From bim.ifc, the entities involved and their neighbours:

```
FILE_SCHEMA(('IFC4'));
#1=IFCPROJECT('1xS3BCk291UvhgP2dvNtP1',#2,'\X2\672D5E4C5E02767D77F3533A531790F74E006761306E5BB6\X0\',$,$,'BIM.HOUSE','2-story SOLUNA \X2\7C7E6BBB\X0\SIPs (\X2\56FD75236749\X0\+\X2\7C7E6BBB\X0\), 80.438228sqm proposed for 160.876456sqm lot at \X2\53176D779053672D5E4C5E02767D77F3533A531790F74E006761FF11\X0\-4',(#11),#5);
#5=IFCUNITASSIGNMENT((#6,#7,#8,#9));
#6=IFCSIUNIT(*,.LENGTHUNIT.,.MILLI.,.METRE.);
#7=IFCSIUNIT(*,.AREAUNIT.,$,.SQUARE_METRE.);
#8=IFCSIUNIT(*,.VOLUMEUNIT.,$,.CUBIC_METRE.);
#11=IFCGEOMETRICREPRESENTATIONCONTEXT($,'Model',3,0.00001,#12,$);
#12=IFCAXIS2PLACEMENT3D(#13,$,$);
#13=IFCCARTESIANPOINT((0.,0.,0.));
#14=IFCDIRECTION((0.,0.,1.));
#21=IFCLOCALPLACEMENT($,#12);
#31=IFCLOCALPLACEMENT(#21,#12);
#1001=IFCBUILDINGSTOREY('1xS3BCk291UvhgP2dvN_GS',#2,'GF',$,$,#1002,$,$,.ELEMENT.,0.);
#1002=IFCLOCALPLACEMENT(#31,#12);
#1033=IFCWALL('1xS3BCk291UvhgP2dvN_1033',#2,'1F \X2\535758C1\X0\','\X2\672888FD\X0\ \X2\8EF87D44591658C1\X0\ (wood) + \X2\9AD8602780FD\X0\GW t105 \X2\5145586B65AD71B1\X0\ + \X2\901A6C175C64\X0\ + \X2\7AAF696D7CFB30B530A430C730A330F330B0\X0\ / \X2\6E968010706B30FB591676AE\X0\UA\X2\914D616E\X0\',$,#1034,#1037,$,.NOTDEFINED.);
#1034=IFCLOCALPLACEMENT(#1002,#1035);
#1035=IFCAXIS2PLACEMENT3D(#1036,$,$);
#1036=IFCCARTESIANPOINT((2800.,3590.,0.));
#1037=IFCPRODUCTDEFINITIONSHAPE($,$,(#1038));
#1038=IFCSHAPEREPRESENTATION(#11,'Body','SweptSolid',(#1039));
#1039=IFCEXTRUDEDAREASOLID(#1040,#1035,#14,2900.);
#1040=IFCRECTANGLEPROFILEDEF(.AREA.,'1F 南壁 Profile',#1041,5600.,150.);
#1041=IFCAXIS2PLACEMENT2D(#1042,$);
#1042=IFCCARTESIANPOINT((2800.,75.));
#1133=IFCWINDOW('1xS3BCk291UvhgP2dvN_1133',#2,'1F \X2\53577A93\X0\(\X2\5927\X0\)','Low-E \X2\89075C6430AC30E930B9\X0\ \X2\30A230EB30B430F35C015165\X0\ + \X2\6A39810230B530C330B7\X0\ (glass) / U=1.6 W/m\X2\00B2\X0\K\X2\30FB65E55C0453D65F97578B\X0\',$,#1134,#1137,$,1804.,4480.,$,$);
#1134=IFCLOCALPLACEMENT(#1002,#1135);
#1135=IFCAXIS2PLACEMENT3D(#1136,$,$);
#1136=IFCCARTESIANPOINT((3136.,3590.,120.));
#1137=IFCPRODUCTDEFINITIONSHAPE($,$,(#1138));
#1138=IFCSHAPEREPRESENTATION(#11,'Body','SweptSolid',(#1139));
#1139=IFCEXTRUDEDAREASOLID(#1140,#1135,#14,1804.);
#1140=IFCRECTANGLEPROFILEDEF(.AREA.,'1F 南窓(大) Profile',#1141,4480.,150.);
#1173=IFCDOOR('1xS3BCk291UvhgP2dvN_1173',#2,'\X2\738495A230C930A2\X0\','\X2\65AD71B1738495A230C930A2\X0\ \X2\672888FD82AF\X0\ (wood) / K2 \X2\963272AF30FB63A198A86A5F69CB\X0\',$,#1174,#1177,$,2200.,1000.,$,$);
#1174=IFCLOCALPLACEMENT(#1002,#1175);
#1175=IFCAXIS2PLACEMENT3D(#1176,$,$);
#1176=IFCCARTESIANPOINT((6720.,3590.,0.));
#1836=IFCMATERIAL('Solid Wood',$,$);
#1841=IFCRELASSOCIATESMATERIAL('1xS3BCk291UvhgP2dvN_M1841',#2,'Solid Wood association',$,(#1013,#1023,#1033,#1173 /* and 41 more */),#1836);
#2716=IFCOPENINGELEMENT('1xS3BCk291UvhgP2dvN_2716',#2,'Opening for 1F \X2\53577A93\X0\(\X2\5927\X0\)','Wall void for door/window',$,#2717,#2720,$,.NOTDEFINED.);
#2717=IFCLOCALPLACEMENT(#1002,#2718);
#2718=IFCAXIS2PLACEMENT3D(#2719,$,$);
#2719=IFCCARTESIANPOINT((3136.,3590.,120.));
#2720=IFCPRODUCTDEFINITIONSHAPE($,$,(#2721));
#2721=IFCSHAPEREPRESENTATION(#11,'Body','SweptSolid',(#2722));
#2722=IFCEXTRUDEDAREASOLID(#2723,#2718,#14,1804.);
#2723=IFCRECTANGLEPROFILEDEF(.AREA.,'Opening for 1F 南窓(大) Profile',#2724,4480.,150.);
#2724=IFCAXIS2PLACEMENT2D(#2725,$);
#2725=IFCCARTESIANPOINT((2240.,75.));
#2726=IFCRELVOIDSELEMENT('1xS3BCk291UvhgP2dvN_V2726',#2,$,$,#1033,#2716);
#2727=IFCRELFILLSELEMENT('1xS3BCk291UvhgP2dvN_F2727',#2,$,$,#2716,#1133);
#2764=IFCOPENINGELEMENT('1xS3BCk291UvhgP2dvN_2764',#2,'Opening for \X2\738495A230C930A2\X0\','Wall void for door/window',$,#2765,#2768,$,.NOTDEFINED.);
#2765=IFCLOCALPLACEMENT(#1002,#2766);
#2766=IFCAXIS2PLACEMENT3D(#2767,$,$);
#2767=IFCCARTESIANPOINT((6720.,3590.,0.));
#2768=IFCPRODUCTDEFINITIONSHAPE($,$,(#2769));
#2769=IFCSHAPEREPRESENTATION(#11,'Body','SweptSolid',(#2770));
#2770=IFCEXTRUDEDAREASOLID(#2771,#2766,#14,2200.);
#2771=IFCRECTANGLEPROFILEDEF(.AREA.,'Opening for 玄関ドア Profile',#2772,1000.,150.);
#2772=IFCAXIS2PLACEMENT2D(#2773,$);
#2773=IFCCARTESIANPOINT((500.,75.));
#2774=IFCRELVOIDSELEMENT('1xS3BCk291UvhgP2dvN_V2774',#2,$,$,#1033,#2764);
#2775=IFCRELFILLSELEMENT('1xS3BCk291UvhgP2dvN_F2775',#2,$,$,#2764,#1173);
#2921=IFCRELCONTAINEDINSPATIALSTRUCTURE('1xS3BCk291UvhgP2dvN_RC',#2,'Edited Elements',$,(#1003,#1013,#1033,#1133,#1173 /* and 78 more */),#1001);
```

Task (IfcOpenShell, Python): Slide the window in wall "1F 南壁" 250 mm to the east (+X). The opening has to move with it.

```python
import ifcopenshell
import ifcopenshell.api.geometry
import ifcopenshell.util.placement

model = ifcopenshell.open("bim.ifc")

window = model.by_guid("1xS3BCk291UvhgP2dvN_1133")
opening = window.FillsVoids[0].RelatingOpeningElement
wall = opening.VoidsElements[0].RelatingBuildingElement

wall_matrix = ifcopenshell.util.placement.get_local_placement(wall.ObjectPlacement)
shift = wall_matrix[:3, 0] * 250.0
before = ifcopenshell.util.placement.get_local_placement(window.ObjectPlacement)[:3, 3].copy()

# The window is not placed relative to its opening, so move both.
for product in (opening, window):
    matrix = ifcopenshell.util.placement.get_local_placement(product.ObjectPlacement)
    matrix[:3, 3] += shift
    ifcopenshell.api.geometry.edit_object_placement(model, product=product, matrix=matrix, is_si=False)

after = ifcopenshell.util.placement.get_local_placement(window.ObjectPlacement)[:3, 3]
print("window moved by", (after - before).round(3) + 0.0)

model.write("bim_updated.ifc")
```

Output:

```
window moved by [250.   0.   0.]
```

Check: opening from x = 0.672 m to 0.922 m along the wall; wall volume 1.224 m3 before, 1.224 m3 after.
